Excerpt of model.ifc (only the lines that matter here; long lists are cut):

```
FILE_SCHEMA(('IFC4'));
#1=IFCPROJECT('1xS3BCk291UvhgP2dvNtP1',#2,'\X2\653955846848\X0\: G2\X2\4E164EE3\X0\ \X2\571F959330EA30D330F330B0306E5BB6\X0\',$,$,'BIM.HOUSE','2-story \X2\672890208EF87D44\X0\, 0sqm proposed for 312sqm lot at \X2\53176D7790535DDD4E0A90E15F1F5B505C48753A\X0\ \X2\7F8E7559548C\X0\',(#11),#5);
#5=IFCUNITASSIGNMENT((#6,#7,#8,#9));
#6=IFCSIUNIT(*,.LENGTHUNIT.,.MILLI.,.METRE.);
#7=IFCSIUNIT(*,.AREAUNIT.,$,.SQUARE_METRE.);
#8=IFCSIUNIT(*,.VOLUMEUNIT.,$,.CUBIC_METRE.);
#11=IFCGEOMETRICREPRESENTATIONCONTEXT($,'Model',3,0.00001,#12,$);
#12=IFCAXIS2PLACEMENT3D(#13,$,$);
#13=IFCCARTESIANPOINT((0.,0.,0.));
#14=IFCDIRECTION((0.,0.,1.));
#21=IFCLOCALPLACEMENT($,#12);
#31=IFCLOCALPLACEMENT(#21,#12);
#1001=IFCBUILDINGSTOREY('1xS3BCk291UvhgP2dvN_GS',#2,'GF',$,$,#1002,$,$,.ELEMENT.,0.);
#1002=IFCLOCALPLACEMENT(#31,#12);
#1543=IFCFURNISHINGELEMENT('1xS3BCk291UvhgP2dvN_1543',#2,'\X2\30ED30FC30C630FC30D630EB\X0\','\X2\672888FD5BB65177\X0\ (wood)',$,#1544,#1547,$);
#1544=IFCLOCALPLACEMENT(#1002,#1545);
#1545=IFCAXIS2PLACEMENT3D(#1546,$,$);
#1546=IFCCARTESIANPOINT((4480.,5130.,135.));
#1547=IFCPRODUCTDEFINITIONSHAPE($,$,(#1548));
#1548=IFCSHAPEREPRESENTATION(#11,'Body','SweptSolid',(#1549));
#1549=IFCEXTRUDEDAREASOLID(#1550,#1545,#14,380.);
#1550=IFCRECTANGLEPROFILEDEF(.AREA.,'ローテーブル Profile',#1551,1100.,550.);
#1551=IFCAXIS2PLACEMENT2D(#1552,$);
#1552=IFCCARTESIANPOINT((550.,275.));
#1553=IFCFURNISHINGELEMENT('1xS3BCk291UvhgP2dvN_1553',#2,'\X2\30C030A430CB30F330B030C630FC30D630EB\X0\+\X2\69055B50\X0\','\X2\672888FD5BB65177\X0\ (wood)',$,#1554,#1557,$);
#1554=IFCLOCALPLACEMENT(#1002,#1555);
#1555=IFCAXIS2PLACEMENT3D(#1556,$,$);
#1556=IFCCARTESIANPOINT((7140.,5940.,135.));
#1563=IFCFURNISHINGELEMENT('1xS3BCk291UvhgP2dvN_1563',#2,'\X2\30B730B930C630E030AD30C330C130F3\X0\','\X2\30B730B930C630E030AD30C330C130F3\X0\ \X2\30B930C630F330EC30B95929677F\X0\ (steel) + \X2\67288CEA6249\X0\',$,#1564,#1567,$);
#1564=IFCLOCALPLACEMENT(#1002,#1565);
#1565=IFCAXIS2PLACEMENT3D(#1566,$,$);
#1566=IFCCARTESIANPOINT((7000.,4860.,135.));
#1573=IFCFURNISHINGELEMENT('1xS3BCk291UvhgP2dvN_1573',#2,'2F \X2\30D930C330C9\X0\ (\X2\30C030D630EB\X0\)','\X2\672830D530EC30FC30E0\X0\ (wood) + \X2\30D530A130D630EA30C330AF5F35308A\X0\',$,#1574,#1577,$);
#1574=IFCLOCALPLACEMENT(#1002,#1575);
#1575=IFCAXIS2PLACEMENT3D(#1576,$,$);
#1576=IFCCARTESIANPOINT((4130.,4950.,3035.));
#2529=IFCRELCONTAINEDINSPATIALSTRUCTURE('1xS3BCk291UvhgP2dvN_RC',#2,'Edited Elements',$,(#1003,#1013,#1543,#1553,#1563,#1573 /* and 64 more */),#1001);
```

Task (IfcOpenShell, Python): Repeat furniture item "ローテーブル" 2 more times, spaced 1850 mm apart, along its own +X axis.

```python
import ifcopenshell
import ifcopenshell.api.geometry
import ifcopenshell.api.root
import ifcopenshell.util.element
import ifcopenshell.util.placement

model = ifcopenshell.open("model.ifc")


def reuse_history(source, copy):
    """copy_class also copies each property set's owner history, people and application; keep the originals."""
    for rel in copy.IsDefinedBy:
        if rel.is_a("IfcRelDefinesByProperties") and (history := rel.RelatingPropertyDefinition.OwnerHistory):
            rel.RelatingPropertyDefinition.OwnerHistory = source.OwnerHistory
            ifcopenshell.util.element.remove_deep2(model, history)


source = model.by_id(1543)
base = ifcopenshell.util.placement.get_local_placement(source.ObjectPlacement)
step = base[:3, 0] * 1850.0

for i in range(1, 3):
    copy = ifcopenshell.api.root.copy_class(model, product=source)
    copy.Representation = ifcopenshell.util.element.copy_deep(
        model, source.Representation, exclude=["IfcGeometricRepresentationContext", "IfcRepresentationMap"]
    )
    reuse_history(source, copy)
    matrix = base.copy()
    matrix[:3, 3] += i * step
    print("added at", matrix[:3, 3].round(3) + 0.0)
    ifcopenshell.api.geometry.edit_object_placement(model, product=copy, matrix=matrix, is_si=False)

model.write("model_updated.ifc")
```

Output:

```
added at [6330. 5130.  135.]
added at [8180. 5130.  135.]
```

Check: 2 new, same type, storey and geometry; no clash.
